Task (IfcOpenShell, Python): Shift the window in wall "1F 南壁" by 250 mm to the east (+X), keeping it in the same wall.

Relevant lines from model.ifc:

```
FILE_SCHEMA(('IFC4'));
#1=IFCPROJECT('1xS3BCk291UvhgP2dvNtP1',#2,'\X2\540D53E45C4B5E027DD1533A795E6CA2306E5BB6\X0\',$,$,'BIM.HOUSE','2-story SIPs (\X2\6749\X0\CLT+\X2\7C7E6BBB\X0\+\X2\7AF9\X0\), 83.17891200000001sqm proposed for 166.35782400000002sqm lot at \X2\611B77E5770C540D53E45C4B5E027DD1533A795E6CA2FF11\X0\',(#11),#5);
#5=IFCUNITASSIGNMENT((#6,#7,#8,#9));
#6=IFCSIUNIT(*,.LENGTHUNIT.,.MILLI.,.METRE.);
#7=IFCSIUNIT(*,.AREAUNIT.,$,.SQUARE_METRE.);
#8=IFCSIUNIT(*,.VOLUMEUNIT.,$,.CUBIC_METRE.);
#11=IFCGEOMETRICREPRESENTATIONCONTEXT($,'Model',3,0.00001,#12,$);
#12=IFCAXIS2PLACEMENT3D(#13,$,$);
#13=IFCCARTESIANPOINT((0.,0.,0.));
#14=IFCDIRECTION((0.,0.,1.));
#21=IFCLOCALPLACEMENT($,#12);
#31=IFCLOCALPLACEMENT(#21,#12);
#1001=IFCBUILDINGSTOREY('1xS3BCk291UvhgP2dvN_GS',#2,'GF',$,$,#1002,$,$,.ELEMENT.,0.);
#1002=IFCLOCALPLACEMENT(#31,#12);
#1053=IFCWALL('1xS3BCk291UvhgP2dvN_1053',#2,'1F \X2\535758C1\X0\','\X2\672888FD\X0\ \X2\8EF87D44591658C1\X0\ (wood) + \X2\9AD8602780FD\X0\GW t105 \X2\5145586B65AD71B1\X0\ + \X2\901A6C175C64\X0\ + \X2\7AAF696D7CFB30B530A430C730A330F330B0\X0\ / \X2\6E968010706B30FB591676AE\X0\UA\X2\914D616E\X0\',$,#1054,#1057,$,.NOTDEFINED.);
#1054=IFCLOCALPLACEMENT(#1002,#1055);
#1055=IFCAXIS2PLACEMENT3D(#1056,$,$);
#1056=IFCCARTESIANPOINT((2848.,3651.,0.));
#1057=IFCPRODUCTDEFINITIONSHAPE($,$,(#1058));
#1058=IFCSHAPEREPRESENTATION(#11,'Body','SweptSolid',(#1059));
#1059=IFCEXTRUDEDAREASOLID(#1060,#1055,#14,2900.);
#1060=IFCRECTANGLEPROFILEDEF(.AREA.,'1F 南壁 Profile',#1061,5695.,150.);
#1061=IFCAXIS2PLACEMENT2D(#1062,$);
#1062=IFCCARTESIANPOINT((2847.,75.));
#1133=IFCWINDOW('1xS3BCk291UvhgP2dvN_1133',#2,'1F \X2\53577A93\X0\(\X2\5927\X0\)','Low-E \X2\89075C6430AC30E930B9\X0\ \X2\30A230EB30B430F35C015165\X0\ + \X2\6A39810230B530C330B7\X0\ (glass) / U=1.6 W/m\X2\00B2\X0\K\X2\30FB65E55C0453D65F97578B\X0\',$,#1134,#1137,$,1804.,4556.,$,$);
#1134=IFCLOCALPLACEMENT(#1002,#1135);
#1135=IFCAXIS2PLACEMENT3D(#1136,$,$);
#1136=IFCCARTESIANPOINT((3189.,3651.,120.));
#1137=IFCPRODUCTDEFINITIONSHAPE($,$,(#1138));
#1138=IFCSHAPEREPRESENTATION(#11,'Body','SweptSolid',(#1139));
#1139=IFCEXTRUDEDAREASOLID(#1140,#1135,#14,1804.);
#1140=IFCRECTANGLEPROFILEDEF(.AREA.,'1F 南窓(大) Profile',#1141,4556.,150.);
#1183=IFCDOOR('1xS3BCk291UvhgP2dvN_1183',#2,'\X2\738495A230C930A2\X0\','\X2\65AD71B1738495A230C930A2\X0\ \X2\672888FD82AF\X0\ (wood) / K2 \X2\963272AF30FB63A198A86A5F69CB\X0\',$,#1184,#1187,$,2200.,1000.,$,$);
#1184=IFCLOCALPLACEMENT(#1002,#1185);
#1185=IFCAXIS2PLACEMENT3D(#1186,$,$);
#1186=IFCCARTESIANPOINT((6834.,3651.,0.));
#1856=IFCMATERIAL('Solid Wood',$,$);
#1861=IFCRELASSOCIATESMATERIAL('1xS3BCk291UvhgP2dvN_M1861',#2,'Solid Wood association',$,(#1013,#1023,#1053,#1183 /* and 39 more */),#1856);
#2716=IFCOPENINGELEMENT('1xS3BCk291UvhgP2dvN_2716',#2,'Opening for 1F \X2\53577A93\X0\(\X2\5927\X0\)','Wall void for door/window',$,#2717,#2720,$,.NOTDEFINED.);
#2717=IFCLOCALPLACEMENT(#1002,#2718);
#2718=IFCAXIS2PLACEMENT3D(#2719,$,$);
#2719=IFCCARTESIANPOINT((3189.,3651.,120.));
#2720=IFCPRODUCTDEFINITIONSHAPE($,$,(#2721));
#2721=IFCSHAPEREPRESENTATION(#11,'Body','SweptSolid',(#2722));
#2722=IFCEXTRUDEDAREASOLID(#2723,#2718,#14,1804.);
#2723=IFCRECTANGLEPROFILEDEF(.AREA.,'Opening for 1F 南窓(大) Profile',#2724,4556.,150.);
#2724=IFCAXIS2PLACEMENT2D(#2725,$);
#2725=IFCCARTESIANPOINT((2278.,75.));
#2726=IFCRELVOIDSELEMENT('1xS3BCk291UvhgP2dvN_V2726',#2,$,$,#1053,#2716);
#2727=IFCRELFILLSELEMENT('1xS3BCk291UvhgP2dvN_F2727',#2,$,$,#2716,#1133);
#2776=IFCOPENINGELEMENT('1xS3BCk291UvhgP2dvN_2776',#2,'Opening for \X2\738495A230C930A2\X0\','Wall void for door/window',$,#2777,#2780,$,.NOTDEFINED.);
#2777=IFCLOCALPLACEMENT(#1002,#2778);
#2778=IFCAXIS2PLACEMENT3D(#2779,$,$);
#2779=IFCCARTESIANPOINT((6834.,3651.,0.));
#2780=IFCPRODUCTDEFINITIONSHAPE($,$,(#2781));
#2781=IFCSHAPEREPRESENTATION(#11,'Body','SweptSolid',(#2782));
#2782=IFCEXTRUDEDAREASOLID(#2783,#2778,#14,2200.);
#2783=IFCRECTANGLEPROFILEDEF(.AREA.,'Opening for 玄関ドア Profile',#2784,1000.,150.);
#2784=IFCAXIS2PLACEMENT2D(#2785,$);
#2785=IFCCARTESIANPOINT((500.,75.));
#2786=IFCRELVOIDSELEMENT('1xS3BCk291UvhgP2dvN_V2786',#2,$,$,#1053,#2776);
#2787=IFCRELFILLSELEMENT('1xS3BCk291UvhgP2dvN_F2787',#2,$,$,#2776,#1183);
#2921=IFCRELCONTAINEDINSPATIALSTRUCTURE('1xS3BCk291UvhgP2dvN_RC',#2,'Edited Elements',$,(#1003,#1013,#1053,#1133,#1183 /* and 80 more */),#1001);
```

```python
import ifcopenshell
import ifcopenshell.api.geometry
import ifcopenshell.util.placement
import ifcopenshell.util.unit

model = ifcopenshell.open("model.ifc")
unit_scale = ifcopenshell.util.unit.calculate_unit_scale(model)

window = model.by_id(1133)
opening = window.FillsVoids[0].RelatingOpeningElement
wall = opening.VoidsElements[0].RelatingBuildingElement

wall_matrix = ifcopenshell.util.placement.get_local_placement(wall.ObjectPlacement)
shift = wall_matrix[:3, 0] * 0.25 / unit_scale
before = ifcopenshell.util.placement.get_local_placement(window.ObjectPlacement)[:3, 3].copy()

# The window is not placed relative to its opening, so move both.
for product in (opening, window):
    matrix = ifcopenshell.util.placement.get_local_placement(product.ObjectPlacement)
    matrix[:3, 3] += shift
    ifcopenshell.api.geometry.edit_object_placement(model, product=product, matrix=matrix, is_si=False)

after = ifcopenshell.util.placement.get_local_placement(window.ObjectPlacement)[:3, 3]
print("window moved by", (after - before).round(3) + 0.0)

model.write("model_edited.ifc")
```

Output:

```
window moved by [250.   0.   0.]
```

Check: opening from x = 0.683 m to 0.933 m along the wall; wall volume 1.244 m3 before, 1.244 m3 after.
